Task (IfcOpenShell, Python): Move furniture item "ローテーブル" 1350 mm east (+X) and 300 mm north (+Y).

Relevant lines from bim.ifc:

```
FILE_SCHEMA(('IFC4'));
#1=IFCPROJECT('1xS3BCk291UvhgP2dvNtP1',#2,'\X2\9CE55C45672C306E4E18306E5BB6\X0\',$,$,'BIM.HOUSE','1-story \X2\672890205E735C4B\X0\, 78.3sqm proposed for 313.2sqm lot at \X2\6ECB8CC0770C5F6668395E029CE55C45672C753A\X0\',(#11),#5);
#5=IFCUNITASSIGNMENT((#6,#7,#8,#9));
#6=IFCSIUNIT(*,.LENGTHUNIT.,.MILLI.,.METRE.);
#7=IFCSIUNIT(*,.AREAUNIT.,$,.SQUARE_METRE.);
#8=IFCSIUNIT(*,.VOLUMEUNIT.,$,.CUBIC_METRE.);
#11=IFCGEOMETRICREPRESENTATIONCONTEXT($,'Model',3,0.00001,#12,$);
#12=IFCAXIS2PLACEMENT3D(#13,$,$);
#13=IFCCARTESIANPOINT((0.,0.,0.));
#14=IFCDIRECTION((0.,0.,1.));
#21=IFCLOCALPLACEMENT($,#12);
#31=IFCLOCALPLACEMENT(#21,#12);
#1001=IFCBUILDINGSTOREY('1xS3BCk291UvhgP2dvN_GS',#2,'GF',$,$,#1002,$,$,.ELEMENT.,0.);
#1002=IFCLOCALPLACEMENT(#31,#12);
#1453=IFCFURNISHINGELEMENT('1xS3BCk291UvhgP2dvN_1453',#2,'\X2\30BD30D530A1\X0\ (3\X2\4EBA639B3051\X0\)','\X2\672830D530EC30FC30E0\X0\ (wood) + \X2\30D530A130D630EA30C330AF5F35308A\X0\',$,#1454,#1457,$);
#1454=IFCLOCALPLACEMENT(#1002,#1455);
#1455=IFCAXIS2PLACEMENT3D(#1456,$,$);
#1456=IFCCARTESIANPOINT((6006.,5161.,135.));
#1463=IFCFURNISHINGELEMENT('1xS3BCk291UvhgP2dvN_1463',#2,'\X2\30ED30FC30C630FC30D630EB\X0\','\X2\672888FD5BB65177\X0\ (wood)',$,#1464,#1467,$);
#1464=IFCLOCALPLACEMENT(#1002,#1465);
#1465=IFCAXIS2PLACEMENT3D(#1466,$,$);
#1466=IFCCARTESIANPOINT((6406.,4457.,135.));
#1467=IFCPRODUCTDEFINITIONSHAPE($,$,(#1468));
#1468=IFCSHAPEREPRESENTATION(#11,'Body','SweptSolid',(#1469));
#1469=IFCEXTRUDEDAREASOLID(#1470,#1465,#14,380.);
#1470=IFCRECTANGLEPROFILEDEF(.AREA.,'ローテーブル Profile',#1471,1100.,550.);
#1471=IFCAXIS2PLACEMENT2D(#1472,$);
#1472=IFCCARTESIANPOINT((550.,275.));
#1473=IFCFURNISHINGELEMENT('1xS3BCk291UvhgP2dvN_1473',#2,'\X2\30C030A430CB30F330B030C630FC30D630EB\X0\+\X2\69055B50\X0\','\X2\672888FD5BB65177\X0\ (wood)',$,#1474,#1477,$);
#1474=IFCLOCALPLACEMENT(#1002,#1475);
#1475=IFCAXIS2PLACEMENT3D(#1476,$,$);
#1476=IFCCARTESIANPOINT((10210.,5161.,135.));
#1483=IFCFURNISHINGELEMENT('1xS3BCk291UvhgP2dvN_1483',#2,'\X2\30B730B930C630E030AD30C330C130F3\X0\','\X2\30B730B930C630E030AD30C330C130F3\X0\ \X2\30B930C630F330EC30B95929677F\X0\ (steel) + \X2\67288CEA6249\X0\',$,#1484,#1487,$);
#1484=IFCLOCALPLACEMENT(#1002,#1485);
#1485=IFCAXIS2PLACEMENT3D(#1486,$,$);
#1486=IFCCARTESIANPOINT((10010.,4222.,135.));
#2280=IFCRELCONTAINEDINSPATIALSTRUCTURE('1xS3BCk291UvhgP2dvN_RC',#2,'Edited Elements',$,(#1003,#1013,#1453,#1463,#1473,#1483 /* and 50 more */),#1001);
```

```python
import ifcopenshell
import ifcopenshell.api.geometry
import ifcopenshell.util.placement
import ifcopenshell.util.unit

model = ifcopenshell.open("bim.ifc")
unit_scale = ifcopenshell.util.unit.calculate_unit_scale(model)

item = model.by_guid("1xS3BCk291UvhgP2dvN_1463")
matrix = ifcopenshell.util.placement.get_local_placement(item.ObjectPlacement)
matrix[0, 3] += 1.35 / unit_scale
matrix[1, 3] += 0.3 / unit_scale
ifcopenshell.api.geometry.edit_object_placement(model, product=item, matrix=matrix, is_si=False)

print(ifcopenshell.util.placement.get_local_placement(item.ObjectPlacement).round(3) + 0.0)

model.write("bim_v2.ifc")
```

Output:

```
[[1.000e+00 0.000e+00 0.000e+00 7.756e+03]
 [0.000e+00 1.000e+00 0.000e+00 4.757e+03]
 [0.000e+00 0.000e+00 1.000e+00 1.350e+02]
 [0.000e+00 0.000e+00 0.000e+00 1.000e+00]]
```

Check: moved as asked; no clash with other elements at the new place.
